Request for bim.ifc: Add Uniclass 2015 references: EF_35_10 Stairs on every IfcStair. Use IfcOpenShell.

First a look at what the model holds.

```python
import ifcopenshell

model = ifcopenshell.open("bim.ifc")
print(model.schema)
print("classifications:", [c.Name for c in model.by_type("IfcClassification")])
for ifc_class in ("IfcDoor", "IfcRoof", "IfcStair", "IfcWall", "IfcWindow"):
    print(ifc_class, len(model.by_type(ifc_class)))
```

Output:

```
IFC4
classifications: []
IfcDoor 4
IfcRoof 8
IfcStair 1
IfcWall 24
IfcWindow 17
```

```python
import ifcopenshell
import ifcopenshell.api.classification

model = ifcopenshell.open("bim.ifc")

system = ifcopenshell.api.classification.add_classification(model, classification="Uniclass 2015")

codes = {
    "IfcStair": ("EF_35_10", "Stairs"),
}
for ifc_class, (code, name) in codes.items():
    products = model.by_type(ifc_class)
    ifcopenshell.api.classification.add_reference(
        model, products=products, classification=system, identification=code, name=name
    )
    print(code, len(products))

model.write("bim_edited.ifc")
```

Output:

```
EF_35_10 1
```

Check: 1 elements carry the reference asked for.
